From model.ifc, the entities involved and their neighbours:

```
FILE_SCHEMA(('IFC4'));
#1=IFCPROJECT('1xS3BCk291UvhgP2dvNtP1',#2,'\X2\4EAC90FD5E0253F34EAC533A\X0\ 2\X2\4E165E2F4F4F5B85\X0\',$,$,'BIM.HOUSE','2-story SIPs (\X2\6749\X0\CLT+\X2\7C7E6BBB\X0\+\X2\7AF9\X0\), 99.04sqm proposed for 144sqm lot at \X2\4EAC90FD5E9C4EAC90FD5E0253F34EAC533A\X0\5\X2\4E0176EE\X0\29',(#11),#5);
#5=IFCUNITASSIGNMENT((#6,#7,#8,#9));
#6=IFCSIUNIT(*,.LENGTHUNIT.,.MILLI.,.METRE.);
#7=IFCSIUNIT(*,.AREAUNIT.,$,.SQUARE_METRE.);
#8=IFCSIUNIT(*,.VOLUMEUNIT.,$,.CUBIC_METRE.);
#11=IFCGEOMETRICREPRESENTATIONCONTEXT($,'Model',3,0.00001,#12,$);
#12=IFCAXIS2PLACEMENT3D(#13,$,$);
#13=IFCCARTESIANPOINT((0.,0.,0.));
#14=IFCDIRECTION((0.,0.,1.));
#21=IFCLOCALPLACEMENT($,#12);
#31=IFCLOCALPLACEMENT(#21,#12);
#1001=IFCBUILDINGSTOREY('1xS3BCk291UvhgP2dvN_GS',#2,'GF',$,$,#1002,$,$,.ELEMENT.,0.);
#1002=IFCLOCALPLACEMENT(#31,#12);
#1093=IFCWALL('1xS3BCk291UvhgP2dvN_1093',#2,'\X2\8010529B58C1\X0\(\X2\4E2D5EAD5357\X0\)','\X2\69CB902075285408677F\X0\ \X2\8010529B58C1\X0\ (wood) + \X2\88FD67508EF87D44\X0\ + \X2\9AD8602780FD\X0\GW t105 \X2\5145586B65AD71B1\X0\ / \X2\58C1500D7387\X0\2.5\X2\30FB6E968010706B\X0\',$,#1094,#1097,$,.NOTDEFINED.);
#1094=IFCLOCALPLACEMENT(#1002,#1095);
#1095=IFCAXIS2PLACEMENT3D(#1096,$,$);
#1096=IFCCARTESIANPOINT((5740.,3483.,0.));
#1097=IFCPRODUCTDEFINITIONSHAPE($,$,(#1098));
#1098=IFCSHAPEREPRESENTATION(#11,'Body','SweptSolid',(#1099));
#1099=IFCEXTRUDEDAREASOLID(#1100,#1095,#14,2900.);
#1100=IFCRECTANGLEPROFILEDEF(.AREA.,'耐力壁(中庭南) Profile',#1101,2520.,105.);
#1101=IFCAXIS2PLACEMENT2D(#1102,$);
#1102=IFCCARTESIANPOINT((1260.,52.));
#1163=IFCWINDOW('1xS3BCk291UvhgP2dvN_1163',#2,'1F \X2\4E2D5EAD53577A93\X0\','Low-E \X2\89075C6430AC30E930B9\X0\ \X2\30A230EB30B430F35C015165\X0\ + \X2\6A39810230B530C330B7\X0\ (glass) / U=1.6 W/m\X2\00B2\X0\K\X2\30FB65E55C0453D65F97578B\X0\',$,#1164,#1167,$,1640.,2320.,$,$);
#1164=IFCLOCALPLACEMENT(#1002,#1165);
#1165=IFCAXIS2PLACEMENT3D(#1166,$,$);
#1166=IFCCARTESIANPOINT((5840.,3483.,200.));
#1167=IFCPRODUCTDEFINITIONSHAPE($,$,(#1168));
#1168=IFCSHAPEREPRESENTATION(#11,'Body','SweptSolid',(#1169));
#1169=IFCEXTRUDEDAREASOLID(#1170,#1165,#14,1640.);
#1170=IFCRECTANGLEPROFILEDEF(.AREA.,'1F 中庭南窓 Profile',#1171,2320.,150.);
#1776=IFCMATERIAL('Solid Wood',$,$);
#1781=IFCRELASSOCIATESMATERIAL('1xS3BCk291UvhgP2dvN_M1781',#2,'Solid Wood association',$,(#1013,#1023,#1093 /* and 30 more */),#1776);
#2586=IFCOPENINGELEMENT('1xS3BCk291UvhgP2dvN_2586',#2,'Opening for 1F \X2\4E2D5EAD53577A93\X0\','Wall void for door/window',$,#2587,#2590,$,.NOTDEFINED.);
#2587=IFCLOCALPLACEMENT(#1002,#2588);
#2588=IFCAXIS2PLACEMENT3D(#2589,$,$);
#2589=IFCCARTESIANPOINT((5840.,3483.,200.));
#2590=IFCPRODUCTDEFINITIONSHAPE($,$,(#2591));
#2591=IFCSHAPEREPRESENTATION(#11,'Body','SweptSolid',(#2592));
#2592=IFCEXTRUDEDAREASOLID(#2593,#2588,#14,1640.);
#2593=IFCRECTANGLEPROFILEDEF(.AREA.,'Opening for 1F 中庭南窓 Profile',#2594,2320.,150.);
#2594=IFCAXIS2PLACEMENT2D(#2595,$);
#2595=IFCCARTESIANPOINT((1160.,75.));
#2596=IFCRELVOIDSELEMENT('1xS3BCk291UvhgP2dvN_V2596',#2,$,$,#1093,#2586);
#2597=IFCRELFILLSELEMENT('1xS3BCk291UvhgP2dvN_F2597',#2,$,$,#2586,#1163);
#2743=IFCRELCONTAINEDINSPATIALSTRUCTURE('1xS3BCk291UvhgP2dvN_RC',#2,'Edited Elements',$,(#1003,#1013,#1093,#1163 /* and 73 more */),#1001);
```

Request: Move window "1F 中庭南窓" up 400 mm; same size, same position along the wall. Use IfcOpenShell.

```python
import numpy as np
import ifcopenshell
import ifcopenshell.api.geometry
import ifcopenshell.util.placement
import ifcopenshell.util.unit

model = ifcopenshell.open("model.ifc")
unit_scale = ifcopenshell.util.unit.calculate_unit_scale(model)

window = model.by_guid("1xS3BCk291UvhgP2dvN_1163")
opening = window.FillsVoids[0].RelatingOpeningElement
dz = 400.0

shift = np.array([0.0, 0.0, dz])
# The window is not placed relative to its opening, so move both.
for product in (opening, window):
    matrix = ifcopenshell.util.placement.get_local_placement(product.ObjectPlacement)
    matrix[:3, 3] += shift
    ifcopenshell.api.geometry.edit_object_placement(model, product=product, matrix=matrix, is_si=False)

print(f"moved by {dz * unit_scale:+.3f} m")

model.write("model-out.ifc")
```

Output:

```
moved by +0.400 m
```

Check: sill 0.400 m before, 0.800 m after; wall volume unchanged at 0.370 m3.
